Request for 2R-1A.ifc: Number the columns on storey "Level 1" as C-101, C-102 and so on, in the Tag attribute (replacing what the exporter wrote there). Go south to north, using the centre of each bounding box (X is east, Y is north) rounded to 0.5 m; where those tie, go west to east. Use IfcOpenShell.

First a look at what the model holds.

```python
import ifcopenshell
import ifcopenshell.util.element
import ifcopenshell.util.placement

model = ifcopenshell.open("2R-1A.ifc")
print(model.schema)
storey = next(s for s in model.by_type("IfcBuildingStorey") if s.Name == "Level 1")
columns = [e for e in ifcopenshell.util.element.get_decomposition(storey) if e.is_a("IfcColumn")]
for e in sorted(columns, key=lambda e: e.id()):
    origin = ifcopenshell.util.placement.get_local_placement(e.ObjectPlacement)[:3, 3]
    print(e.id(), e.Tag, e.Name, origin.round(2) + 0.0, sep=" | ")
```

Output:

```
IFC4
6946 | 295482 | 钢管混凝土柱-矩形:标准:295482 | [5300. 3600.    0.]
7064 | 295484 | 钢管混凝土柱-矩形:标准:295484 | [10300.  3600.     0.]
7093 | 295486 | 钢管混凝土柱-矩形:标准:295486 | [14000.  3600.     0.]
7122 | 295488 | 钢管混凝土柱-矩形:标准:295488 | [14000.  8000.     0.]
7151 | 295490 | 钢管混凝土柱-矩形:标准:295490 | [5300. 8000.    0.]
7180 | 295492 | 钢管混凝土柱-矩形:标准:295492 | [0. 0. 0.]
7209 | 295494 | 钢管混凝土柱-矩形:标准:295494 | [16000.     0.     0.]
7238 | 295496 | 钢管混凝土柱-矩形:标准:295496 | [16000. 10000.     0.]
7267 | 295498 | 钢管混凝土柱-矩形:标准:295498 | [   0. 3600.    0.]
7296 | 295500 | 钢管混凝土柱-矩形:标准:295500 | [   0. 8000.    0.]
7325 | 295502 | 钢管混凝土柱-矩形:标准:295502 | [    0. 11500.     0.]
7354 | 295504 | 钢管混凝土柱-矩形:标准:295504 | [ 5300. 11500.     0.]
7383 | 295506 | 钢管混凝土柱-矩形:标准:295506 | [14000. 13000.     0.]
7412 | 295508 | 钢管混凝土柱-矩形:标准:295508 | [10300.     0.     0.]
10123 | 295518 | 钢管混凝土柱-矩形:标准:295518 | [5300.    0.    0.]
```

```python
import ifcopenshell
import ifcopenshell.geom
import ifcopenshell.util.element
import ifcopenshell.util.shape

model = ifcopenshell.open("2R-1A.ifc")
settings = ifcopenshell.geom.settings()
settings.set("use-world-coords", True)


def centre(element):
    shape = ifcopenshell.geom.create_shape(settings, element)
    return ifcopenshell.util.shape.get_bbox_centroid(shape.geometry)


storey = next(s for s in model.by_type("IfcBuildingStorey") if s.Name == "Level 1")
columns = [e for e in ifcopenshell.util.element.get_decomposition(storey) if e.is_a("IfcColumn")]

# Insertion points can sit at a corner or the storey origin, so sort by the geometry (in metres).
centres = {e: centre(e) for e in columns}
columns.sort(key=lambda e: (round(centres[e][1] / 0.5), centres[e][0]))

for i, e in enumerate(columns, start=1):
    number = f"C-1{i:02d}"
    e.Tag = number
    print(e.id(), number)

model.write("2R-1A_v2.ifc")
```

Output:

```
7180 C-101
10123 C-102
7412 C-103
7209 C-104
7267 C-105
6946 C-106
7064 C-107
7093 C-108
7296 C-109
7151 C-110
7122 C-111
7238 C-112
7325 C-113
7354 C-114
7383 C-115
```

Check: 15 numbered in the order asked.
